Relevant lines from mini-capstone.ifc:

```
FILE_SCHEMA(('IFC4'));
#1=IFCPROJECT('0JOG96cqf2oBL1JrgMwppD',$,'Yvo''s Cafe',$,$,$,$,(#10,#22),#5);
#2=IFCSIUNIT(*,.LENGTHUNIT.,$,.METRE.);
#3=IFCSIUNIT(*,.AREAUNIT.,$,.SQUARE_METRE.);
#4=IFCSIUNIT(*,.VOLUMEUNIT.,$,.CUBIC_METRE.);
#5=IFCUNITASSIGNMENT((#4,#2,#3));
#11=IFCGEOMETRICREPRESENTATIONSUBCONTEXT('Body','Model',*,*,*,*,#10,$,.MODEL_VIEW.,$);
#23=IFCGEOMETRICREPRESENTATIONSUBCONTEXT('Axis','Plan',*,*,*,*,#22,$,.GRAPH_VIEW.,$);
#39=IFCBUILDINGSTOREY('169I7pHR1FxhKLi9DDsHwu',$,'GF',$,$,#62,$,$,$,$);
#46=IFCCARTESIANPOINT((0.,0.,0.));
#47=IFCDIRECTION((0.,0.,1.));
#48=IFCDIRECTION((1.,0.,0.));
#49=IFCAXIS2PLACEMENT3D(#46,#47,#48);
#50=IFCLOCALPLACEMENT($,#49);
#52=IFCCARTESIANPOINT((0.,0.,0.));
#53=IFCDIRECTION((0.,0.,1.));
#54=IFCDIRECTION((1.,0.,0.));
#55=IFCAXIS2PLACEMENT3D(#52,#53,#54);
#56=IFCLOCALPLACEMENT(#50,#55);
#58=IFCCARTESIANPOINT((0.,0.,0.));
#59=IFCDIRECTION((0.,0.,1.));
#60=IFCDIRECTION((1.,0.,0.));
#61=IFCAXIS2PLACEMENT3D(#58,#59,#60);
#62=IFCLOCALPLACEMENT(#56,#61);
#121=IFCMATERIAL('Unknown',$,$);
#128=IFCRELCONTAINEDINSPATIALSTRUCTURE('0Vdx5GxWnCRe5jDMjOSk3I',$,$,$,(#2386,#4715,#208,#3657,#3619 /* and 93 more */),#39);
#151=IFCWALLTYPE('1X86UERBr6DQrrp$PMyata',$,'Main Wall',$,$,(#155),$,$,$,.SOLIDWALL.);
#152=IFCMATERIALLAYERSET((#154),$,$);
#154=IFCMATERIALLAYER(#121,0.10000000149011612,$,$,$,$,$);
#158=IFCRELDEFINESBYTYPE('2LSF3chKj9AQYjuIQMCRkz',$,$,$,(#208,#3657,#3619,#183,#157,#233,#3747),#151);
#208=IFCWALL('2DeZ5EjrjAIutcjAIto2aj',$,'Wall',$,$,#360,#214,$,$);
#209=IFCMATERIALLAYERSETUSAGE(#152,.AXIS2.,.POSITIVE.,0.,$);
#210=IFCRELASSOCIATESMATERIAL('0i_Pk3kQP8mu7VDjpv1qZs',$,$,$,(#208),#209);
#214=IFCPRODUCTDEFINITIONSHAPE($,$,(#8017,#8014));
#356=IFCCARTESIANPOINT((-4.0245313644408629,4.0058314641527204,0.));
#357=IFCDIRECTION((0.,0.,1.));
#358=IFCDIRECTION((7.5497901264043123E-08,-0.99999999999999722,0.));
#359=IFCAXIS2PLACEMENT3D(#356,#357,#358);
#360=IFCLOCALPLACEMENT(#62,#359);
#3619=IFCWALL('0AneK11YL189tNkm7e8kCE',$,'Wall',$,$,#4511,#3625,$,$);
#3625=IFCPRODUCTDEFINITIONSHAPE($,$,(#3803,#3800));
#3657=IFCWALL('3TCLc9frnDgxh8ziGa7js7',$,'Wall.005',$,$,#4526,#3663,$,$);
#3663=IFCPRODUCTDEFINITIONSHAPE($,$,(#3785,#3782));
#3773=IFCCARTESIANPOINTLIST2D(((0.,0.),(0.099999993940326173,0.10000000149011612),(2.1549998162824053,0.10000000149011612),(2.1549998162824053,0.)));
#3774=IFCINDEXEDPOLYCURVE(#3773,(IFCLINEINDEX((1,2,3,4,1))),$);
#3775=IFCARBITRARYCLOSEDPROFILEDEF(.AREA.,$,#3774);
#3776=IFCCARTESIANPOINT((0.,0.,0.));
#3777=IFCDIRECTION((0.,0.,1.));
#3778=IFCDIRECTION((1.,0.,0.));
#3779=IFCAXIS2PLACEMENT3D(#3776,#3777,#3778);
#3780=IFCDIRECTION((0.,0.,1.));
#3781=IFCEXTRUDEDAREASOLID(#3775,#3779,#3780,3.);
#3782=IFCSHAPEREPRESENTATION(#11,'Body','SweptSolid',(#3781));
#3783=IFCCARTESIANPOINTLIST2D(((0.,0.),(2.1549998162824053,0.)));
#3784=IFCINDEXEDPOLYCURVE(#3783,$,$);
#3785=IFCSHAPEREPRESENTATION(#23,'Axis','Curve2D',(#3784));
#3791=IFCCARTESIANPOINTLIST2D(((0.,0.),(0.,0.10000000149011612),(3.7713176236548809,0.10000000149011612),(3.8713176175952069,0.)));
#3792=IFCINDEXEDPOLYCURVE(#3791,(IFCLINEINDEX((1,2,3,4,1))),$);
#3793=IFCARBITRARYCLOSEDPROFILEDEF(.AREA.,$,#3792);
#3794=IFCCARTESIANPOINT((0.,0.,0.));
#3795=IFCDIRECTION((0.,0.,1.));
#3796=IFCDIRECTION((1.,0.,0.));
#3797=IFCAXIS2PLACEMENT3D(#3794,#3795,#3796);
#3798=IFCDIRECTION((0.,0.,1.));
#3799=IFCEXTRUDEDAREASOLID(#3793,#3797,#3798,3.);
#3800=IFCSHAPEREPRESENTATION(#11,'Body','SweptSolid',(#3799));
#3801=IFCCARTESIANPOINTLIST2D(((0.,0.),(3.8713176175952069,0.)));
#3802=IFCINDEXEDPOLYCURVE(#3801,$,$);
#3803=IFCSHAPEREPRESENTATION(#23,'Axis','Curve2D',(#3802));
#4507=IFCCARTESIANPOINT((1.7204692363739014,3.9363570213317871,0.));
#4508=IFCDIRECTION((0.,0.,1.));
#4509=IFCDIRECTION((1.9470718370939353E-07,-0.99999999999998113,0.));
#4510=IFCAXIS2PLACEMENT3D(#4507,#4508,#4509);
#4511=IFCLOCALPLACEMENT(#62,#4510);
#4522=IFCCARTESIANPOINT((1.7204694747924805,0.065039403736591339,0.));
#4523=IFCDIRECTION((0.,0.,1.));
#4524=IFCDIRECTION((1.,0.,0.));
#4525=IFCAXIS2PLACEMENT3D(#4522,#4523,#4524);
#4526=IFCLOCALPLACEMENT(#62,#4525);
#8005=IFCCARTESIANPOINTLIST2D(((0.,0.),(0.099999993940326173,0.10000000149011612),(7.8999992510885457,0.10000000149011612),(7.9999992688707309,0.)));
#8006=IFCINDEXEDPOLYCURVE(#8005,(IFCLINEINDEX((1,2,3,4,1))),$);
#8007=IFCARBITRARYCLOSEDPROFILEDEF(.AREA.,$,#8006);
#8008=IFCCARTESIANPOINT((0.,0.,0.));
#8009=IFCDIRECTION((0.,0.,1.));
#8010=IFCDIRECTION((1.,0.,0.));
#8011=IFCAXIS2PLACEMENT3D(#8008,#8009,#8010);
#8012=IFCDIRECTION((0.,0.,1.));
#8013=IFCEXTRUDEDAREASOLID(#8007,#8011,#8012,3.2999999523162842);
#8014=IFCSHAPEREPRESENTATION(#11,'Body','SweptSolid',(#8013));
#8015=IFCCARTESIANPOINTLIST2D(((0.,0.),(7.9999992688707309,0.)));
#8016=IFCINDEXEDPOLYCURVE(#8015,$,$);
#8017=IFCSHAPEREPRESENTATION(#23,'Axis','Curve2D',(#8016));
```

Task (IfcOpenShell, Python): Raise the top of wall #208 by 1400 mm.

```python
import ifcopenshell
import ifcopenshell.geom
import ifcopenshell.util.representation
import ifcopenshell.util.shape

model = ifcopenshell.open("mini-capstone.ifc")
settings = ifcopenshell.geom.settings()


def volume(element):
    """Net volume in cubic metres, openings subtracted."""
    shape = ifcopenshell.geom.create_shape(settings, element)
    return ifcopenshell.util.shape.get_volume(shape.geometry)


wall = model.by_id(208)
before = volume(wall)

body = ifcopenshell.util.representation.get_representation(wall, "Model", "Body")
solid = body.Items[0]
old_height = solid.Depth
solid.Depth += 1.4
after = volume(wall)

print(f"height {old_height:g} -> {solid.Depth:g}, volume {before:.3f} -> {after:.3f} m3")

model.write("mini-capstone_updated.ifc")
```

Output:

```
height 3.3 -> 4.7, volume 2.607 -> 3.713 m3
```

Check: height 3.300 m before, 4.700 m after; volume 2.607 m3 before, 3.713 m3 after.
